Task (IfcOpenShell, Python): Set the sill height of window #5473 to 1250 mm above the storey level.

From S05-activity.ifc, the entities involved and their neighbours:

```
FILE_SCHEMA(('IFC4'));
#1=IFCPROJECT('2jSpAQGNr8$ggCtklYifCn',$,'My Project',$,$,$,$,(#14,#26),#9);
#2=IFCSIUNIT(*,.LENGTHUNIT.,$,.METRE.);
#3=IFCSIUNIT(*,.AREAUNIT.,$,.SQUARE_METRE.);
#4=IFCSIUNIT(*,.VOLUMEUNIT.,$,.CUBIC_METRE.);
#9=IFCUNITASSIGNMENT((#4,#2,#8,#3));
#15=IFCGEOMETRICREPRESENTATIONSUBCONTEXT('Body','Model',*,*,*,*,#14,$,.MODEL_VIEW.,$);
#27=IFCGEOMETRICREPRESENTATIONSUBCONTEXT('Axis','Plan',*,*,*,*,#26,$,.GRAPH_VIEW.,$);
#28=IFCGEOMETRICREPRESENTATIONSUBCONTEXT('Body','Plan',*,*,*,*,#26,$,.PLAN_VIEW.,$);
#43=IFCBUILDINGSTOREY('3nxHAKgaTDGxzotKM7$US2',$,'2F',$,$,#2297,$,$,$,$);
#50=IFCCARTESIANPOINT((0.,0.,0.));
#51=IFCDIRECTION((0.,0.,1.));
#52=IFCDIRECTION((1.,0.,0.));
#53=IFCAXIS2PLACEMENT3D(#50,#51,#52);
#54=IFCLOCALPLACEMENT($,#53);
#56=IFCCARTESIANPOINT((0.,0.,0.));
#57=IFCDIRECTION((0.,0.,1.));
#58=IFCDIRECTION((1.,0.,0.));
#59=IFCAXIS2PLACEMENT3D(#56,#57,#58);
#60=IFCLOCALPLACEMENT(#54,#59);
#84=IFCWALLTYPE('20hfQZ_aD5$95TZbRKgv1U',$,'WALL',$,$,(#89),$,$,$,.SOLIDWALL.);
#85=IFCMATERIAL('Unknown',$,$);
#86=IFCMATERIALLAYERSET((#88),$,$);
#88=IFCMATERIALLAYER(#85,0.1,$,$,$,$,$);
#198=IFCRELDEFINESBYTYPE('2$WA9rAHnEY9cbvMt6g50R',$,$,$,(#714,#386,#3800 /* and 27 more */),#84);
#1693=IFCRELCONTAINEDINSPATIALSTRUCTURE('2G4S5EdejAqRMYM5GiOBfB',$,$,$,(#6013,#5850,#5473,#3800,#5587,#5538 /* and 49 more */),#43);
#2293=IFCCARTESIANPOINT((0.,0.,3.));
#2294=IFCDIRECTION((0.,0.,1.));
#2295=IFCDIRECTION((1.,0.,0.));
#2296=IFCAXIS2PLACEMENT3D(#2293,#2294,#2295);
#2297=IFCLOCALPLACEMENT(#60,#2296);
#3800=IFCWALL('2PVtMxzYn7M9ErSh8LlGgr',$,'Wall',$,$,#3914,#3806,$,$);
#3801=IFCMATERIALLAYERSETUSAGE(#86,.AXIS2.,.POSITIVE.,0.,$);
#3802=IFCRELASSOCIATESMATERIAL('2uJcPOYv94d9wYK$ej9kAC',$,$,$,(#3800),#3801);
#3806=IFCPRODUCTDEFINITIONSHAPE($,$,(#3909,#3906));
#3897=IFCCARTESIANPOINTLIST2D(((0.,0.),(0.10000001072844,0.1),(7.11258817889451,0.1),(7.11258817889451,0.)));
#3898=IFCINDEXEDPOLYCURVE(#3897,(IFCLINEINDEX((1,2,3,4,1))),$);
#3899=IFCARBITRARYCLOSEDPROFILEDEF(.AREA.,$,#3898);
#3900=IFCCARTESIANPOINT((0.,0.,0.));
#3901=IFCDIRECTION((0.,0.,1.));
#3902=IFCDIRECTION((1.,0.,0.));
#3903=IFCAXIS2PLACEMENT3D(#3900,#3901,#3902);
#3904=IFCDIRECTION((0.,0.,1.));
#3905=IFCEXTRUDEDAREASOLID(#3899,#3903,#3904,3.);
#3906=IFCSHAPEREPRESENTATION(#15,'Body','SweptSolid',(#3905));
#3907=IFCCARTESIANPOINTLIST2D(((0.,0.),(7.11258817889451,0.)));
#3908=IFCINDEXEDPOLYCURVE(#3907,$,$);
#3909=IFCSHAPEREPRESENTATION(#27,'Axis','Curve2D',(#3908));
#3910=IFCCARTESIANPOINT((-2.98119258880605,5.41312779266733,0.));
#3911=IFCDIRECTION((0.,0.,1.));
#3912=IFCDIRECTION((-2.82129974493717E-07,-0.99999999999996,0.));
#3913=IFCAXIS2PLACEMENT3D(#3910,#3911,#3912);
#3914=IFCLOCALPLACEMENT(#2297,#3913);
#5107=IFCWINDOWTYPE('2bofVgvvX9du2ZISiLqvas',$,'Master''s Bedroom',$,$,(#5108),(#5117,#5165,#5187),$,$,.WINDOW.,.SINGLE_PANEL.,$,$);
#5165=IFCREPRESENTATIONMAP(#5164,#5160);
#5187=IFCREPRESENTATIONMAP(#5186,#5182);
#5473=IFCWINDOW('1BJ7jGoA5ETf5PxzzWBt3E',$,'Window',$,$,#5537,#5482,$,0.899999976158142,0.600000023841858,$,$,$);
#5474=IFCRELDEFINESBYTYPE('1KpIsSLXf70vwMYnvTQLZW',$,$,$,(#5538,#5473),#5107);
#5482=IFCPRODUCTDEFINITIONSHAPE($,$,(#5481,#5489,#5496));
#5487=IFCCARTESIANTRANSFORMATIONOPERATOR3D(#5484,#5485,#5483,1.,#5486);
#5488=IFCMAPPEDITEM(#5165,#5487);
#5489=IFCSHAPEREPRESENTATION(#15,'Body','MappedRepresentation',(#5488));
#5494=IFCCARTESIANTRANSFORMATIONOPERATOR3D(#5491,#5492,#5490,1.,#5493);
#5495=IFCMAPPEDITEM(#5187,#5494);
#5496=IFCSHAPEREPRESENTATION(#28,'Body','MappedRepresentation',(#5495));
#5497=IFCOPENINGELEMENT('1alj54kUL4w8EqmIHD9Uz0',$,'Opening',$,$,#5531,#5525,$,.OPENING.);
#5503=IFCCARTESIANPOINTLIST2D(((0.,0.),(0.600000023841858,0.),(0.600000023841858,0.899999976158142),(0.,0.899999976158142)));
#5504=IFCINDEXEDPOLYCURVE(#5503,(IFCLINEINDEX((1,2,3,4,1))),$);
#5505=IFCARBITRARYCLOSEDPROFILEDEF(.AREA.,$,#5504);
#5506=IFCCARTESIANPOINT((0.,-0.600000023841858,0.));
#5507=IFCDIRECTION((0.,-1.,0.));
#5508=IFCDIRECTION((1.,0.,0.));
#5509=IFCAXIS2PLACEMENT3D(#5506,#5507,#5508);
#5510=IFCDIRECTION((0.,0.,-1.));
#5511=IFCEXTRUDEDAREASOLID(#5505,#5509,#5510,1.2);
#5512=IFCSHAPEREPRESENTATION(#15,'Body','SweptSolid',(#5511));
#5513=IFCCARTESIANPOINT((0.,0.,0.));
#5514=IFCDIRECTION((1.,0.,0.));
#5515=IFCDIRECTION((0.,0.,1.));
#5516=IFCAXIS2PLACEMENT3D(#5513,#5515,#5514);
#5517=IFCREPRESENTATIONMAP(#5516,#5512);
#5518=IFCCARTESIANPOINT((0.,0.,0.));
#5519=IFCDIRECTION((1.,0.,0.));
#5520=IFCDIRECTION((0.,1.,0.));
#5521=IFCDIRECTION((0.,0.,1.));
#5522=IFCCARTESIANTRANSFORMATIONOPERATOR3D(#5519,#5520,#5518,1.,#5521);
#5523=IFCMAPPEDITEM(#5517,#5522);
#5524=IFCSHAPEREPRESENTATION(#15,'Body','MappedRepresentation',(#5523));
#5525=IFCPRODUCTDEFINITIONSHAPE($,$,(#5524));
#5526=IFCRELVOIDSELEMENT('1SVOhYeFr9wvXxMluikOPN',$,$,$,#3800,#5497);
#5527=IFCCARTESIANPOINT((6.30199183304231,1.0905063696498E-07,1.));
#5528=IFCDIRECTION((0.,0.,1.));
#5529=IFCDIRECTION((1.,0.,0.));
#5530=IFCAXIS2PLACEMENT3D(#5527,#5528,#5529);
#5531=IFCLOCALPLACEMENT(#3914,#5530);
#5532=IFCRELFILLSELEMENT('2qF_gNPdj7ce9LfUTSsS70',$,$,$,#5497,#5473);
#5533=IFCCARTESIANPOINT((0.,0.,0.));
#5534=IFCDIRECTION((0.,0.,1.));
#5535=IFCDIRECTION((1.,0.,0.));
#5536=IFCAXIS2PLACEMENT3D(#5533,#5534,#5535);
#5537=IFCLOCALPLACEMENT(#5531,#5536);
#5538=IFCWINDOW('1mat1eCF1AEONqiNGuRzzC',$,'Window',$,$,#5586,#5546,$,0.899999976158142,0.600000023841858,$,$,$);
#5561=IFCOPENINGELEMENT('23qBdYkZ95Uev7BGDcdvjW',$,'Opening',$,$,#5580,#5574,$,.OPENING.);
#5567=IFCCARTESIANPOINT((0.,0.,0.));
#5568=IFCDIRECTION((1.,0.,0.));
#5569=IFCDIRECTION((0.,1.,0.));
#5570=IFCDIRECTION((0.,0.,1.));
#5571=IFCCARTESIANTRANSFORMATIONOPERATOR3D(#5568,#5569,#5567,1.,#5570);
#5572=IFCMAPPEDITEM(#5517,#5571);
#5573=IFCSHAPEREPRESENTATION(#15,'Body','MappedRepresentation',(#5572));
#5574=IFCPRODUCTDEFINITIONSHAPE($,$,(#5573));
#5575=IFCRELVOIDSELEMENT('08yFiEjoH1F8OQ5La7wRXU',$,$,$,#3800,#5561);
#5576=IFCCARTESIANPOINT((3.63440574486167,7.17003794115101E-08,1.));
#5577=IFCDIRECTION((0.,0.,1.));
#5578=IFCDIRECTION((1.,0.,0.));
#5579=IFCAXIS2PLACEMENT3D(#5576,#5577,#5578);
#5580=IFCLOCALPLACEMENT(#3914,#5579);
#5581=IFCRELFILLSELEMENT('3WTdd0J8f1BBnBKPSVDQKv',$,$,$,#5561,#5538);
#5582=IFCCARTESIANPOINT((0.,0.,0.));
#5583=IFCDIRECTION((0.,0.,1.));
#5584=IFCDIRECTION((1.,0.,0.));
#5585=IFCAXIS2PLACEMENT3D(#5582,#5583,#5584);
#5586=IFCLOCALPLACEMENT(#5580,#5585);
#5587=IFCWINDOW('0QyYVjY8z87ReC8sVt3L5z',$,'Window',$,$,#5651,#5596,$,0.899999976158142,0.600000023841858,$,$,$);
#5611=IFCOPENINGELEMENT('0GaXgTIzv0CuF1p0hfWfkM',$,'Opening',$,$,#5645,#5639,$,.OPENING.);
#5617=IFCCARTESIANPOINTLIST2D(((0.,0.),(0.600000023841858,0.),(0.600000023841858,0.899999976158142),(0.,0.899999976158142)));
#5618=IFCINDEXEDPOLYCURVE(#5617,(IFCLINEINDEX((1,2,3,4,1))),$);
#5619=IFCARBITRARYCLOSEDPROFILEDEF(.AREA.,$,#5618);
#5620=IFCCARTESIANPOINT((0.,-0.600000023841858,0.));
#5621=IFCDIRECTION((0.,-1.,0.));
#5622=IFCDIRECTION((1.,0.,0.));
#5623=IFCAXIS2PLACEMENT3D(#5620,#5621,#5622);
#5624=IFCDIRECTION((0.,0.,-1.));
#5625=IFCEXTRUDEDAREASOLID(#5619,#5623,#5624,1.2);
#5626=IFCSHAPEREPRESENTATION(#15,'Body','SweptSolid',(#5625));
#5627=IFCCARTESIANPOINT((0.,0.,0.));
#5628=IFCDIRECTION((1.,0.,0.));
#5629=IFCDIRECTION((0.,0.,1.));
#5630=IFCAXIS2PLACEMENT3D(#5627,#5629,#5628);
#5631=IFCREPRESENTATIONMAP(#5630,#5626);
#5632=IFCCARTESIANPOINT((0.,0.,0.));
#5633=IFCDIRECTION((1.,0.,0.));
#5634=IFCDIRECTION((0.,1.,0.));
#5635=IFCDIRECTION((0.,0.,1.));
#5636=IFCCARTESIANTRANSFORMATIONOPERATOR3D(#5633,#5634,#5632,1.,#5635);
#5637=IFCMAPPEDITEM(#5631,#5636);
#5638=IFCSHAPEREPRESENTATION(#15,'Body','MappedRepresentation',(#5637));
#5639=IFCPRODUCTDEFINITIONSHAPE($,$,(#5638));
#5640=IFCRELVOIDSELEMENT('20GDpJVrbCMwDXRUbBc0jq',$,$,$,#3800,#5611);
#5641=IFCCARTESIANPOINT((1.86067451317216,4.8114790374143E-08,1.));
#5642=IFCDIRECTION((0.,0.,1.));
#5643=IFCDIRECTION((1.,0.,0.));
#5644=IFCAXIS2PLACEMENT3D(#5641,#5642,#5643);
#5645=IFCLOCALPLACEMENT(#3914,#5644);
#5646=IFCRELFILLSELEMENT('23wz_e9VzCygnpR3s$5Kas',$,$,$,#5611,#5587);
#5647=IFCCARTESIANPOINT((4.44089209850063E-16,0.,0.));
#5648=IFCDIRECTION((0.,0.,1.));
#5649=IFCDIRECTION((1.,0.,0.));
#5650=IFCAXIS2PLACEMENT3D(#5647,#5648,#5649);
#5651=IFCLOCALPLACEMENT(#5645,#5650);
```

```python
import numpy as np
import ifcopenshell
import ifcopenshell.api.geometry
import ifcopenshell.geom
import ifcopenshell.util.element
import ifcopenshell.util.placement
import ifcopenshell.util.shape
import ifcopenshell.util.unit

model = ifcopenshell.open("S05-activity.ifc")
unit_scale = ifcopenshell.util.unit.calculate_unit_scale(model)

window = model.by_guid("1BJ7jGoA5ETf5PxzzWBt3E")
opening = window.FillsVoids[0].RelatingOpeningElement
storey = ifcopenshell.util.element.get_container(window, ifc_class="IfcBuildingStorey")
level = ifcopenshell.util.placement.get_local_placement(storey.ObjectPlacement)[2, 3]

# The opening's origin need not be at the sill, so measure its lowest point.
shape = ifcopenshell.geom.create_shape(ifcopenshell.geom.settings(), opening)
bottom = ifcopenshell.util.shape.get_shape_bottom_elevation(shape, shape.geometry) / unit_scale
dz = level + 1.25 / unit_scale - bottom

shift = np.array([0.0, 0.0, dz])
# The window is placed relative to its opening, so it follows when the opening moves.
matrix = ifcopenshell.util.placement.get_local_placement(opening.ObjectPlacement)
matrix[:3, 3] += shift
ifcopenshell.api.geometry.edit_object_placement(
    model, product=opening, matrix=matrix, is_si=False, should_transform_children=True
)

print(f"moved by {dz * unit_scale:+.3f} m")

model.write("S05-activity_rev.ifc")
```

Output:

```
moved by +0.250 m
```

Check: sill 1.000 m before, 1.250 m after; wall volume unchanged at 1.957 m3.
